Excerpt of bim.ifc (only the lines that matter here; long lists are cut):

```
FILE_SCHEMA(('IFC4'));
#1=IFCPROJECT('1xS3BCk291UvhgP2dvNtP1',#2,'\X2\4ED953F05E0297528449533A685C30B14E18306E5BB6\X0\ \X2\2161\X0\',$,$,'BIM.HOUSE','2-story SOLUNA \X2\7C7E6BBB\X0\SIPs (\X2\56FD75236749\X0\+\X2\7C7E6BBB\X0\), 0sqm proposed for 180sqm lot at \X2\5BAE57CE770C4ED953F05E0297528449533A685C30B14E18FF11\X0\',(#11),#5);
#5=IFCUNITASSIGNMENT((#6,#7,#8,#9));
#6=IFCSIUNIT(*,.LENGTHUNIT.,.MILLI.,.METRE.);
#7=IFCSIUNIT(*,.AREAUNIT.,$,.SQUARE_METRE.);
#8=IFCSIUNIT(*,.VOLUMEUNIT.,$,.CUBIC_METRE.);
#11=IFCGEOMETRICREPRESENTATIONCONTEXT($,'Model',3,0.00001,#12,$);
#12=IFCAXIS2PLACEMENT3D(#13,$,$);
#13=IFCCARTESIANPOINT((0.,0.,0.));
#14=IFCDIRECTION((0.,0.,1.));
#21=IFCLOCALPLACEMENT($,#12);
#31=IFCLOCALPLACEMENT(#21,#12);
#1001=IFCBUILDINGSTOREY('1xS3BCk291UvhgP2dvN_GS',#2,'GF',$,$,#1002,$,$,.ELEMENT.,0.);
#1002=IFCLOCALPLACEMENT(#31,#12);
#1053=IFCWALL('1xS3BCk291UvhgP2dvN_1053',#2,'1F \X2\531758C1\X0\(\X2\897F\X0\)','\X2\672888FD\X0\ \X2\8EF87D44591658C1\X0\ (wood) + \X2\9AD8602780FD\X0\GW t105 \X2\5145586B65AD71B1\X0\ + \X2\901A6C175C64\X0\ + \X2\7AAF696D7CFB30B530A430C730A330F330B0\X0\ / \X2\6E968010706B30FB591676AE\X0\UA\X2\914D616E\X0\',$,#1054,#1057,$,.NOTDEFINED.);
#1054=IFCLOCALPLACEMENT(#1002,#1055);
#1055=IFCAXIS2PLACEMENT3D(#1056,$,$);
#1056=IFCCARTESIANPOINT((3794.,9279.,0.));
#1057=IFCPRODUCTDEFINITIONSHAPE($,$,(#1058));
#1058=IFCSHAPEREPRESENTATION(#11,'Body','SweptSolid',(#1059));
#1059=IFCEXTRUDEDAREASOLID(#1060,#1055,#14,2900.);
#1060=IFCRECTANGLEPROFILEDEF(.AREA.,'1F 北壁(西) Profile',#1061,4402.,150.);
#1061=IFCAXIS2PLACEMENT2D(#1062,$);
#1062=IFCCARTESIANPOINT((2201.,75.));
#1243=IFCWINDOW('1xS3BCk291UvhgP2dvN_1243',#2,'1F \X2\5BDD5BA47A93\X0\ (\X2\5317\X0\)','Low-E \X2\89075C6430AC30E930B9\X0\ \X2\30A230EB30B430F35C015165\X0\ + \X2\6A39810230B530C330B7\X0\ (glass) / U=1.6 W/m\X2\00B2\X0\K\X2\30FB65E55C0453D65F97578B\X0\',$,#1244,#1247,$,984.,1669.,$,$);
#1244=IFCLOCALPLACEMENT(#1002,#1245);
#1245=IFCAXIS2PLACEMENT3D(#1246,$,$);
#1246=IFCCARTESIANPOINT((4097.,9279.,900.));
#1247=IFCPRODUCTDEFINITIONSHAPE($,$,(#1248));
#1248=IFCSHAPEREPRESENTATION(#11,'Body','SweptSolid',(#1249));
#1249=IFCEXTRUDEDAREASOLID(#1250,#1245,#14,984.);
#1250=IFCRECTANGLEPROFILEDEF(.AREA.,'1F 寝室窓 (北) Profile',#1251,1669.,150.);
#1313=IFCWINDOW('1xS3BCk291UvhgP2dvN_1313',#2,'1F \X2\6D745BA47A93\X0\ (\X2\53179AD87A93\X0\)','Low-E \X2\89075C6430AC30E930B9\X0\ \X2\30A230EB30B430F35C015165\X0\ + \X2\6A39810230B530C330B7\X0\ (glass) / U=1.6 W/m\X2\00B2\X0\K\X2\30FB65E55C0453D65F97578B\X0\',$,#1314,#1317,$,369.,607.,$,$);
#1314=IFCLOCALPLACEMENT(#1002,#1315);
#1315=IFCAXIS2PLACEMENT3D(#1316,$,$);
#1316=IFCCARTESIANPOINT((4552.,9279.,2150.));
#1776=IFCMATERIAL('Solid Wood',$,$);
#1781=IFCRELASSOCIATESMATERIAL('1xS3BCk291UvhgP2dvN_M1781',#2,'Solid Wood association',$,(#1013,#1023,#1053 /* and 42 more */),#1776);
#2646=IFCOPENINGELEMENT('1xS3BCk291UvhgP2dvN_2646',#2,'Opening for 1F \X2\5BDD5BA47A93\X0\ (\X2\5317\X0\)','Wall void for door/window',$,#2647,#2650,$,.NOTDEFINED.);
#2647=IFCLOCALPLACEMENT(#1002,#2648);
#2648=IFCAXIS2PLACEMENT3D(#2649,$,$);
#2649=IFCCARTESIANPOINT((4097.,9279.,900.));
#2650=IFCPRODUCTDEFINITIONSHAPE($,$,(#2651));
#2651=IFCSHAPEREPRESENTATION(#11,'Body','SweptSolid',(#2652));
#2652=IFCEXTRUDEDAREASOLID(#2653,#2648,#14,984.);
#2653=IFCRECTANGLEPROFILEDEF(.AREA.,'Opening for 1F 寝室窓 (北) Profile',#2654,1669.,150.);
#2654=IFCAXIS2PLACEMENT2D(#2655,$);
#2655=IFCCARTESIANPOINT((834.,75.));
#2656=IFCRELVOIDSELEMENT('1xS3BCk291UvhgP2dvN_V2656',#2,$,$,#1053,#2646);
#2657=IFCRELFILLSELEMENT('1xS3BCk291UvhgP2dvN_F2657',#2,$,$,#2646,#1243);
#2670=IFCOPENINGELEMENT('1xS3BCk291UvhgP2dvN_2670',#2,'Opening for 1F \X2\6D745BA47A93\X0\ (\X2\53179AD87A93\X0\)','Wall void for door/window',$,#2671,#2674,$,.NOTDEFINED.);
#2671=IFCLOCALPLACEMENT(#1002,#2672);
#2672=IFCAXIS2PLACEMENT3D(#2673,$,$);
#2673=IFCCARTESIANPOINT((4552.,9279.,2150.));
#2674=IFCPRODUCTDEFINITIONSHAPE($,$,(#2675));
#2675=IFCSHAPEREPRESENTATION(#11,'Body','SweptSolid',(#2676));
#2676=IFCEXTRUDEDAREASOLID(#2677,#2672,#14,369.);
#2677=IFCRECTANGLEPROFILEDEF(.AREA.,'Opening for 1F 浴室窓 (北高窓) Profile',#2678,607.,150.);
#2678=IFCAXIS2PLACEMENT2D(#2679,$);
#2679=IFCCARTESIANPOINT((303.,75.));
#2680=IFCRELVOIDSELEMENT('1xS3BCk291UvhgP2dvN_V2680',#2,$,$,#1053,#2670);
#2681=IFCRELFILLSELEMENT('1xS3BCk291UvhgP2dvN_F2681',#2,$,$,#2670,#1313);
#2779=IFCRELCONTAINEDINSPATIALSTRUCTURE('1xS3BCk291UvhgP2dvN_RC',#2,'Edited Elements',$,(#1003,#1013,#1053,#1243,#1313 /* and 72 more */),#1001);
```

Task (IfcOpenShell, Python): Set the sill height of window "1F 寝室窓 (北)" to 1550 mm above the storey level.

```python
import numpy as np
import ifcopenshell
import ifcopenshell.api.geometry
import ifcopenshell.geom
import ifcopenshell.util.element
import ifcopenshell.util.placement
import ifcopenshell.util.shape
import ifcopenshell.util.unit

model = ifcopenshell.open("bim.ifc")
unit_scale = ifcopenshell.util.unit.calculate_unit_scale(model)

window = model.by_guid("1xS3BCk291UvhgP2dvN_1243")
opening = window.FillsVoids[0].RelatingOpeningElement
storey = ifcopenshell.util.element.get_container(window, ifc_class="IfcBuildingStorey")
level = ifcopenshell.util.placement.get_local_placement(storey.ObjectPlacement)[2, 3]

# The opening's origin need not be at the sill, so measure its lowest point.
shape = ifcopenshell.geom.create_shape(ifcopenshell.geom.settings(), opening)
bottom = ifcopenshell.util.shape.get_shape_bottom_elevation(shape, shape.geometry) / unit_scale
dz = level + 1.55 / unit_scale - bottom

shift = np.array([0.0, 0.0, dz])
# The window is not placed relative to its opening, so move both.
for product in (opening, window):
    matrix = ifcopenshell.util.placement.get_local_placement(product.ObjectPlacement)
    matrix[:3, 3] += shift
    ifcopenshell.api.geometry.edit_object_placement(model, product=product, matrix=matrix, is_si=False)

print(f"moved by {dz * unit_scale:+.3f} m")

model.write("bim_rev.ifc")
```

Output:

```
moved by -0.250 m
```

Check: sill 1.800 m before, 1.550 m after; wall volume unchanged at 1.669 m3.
